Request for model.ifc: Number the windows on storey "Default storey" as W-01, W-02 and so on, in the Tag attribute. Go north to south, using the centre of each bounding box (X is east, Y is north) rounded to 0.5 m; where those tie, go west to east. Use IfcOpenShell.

First a look at what the model holds.

```python
import ifcopenshell
import ifcopenshell.util.element
import ifcopenshell.util.placement

model = ifcopenshell.open("model.ifc")
print(model.schema)
storey = next(s for s in model.by_type("IfcBuildingStorey") if s.Name == "Default storey")
windows = [e for e in ifcopenshell.util.element.get_decomposition(storey) if e.is_a("IfcWindow")]
for e in sorted(windows, key=lambda e: e.id()):
    origin = ifcopenshell.util.placement.get_local_placement(e.ObjectPlacement)[:3, 3]
    print(e.id(), e.Tag, e.Name, origin.round(2) + 0.0, sep=" | ")
```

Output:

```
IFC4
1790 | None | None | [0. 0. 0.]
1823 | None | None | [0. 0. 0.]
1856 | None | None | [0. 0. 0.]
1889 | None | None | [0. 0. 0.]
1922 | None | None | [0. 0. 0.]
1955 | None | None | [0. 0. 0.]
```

```python
import ifcopenshell
import ifcopenshell.geom
import ifcopenshell.util.element
import ifcopenshell.util.shape

model = ifcopenshell.open("model.ifc")
settings = ifcopenshell.geom.settings()
settings.set("use-world-coords", True)


def centre(element):
    shape = ifcopenshell.geom.create_shape(settings, element)
    return ifcopenshell.util.shape.get_bbox_centroid(shape.geometry)


storey = next(s for s in model.by_type("IfcBuildingStorey") if s.Name == "Default storey")
windows = [e for e in ifcopenshell.util.element.get_decomposition(storey) if e.is_a("IfcWindow")]

# Insertion points can sit at a corner or the storey origin, so sort by the geometry (in metres).
centres = {e: centre(e) for e in windows}
windows.sort(key=lambda e: (-round(centres[e][1] / 0.5), centres[e][0]))

for i, e in enumerate(windows, start=1):
    number = f"W-{i:02d}"
    e.Tag = number
    print(e.id(), number)

model.write("model_v2.ifc")
```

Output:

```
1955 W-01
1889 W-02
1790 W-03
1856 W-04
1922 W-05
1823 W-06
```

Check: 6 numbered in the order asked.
